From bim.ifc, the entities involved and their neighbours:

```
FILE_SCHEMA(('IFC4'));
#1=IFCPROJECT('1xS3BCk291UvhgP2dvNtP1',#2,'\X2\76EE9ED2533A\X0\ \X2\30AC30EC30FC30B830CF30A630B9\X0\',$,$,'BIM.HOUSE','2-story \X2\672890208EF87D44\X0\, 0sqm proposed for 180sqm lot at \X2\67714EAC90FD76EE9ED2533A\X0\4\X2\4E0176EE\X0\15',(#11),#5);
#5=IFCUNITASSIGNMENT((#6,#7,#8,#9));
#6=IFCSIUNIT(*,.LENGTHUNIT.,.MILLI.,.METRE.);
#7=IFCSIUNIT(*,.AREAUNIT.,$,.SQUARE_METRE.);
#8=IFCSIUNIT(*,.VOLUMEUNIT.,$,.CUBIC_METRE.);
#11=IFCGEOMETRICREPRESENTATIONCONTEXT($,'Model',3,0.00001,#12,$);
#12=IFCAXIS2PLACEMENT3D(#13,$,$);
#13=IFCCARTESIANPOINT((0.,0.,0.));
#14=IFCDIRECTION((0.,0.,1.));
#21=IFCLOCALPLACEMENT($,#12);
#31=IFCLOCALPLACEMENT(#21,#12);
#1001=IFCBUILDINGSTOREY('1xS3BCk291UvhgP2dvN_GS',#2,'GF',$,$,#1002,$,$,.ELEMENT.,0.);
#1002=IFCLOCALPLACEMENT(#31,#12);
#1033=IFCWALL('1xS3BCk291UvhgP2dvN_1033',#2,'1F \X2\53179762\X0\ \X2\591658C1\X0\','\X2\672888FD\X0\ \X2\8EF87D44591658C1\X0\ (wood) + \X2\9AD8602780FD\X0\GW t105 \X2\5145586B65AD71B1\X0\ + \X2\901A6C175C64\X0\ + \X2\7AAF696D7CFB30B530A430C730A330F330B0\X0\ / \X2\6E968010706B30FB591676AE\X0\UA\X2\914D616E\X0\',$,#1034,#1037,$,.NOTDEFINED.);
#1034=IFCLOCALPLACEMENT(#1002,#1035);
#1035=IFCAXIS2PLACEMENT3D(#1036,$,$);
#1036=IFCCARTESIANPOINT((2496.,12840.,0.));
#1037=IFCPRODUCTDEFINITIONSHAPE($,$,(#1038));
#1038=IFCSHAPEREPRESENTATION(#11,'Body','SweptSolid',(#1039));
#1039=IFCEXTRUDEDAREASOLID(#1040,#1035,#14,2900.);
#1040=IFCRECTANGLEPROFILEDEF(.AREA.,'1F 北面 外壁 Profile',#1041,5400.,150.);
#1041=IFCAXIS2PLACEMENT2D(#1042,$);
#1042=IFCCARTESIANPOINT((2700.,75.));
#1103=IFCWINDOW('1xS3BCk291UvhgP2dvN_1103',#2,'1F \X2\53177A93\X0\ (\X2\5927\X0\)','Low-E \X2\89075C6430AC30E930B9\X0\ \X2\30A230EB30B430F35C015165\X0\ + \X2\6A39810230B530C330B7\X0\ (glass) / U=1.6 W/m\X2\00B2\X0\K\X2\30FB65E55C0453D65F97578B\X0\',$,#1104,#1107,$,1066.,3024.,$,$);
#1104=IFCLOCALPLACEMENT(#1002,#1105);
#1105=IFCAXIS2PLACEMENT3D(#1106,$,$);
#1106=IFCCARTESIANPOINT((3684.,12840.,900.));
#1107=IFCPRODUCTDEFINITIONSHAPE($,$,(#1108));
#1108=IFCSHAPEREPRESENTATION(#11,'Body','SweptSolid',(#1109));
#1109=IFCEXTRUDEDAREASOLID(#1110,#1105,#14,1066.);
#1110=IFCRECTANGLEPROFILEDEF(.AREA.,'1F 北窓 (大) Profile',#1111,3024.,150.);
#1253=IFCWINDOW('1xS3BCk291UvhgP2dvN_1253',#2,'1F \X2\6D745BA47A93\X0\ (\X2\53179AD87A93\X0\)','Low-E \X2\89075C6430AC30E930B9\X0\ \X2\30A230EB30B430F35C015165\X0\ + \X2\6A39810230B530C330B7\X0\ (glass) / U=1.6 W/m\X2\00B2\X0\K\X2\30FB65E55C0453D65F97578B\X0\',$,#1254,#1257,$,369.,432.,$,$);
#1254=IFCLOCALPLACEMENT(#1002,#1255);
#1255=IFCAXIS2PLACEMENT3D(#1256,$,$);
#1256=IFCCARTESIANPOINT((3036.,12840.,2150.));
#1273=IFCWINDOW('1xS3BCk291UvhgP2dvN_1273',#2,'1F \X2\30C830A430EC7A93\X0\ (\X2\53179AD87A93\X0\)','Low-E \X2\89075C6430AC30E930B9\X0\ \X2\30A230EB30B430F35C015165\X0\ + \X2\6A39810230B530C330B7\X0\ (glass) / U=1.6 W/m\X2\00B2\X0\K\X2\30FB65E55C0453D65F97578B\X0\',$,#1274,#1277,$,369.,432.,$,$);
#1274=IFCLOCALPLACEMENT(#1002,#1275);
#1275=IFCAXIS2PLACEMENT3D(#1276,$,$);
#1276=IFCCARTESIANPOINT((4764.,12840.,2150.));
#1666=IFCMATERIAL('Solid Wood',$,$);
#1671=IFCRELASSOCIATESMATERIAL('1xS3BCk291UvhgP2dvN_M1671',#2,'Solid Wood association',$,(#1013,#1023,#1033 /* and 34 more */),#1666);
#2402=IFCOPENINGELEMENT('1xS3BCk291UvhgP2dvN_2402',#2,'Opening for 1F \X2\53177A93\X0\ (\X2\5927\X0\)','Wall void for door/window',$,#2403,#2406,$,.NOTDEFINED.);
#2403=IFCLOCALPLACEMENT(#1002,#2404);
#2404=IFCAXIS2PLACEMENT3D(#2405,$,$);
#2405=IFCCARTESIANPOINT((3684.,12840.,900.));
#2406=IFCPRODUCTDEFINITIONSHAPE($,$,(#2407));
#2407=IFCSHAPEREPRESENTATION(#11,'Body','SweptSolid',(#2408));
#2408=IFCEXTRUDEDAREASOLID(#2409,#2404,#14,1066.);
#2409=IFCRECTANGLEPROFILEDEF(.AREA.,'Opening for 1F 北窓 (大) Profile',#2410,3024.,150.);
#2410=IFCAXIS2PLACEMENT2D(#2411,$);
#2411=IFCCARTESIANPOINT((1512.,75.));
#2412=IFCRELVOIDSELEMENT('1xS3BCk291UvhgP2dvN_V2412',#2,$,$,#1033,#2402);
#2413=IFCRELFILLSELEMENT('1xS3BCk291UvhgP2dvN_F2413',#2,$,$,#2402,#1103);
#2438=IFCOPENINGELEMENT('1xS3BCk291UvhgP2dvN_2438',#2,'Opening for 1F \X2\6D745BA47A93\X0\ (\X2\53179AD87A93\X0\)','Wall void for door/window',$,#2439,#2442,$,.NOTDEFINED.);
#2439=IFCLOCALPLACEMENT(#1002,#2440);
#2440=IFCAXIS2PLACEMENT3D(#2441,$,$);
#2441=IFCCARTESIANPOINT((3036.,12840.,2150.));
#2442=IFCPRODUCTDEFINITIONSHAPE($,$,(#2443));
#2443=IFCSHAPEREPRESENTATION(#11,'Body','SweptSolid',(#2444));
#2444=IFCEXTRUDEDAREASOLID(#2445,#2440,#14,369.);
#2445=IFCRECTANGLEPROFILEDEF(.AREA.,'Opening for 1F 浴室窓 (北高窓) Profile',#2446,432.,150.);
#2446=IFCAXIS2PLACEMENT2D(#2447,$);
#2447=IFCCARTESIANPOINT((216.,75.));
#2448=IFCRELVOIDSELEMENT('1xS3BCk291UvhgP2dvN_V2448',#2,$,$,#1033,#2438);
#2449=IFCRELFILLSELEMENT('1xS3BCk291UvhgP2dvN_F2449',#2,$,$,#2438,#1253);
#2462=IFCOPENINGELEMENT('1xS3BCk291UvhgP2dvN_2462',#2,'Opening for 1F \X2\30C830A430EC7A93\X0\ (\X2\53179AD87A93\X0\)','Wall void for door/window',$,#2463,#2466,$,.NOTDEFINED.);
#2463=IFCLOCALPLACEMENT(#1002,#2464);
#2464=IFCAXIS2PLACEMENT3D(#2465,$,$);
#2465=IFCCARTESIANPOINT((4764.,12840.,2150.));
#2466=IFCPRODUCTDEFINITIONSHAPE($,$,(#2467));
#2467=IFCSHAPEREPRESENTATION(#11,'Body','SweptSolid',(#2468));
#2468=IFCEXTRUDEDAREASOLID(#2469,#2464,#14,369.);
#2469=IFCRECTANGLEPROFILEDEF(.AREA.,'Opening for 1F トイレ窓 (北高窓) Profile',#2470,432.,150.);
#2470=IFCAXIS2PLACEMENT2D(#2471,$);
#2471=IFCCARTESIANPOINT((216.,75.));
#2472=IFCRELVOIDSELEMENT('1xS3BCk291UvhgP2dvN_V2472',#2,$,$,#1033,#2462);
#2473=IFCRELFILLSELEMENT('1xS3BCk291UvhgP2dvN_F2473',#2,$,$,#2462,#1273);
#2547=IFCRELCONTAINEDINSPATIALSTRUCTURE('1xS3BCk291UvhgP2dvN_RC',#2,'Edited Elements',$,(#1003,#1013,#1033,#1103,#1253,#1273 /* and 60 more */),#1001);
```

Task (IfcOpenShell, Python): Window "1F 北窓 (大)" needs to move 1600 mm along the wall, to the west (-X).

```python
import ifcopenshell
import ifcopenshell.api.geometry
import ifcopenshell.util.placement
import ifcopenshell.util.unit

model = ifcopenshell.open("bim.ifc")
unit_scale = ifcopenshell.util.unit.calculate_unit_scale(model)

window = model.by_guid("1xS3BCk291UvhgP2dvN_1103")
opening = window.FillsVoids[0].RelatingOpeningElement
wall = opening.VoidsElements[0].RelatingBuildingElement

wall_matrix = ifcopenshell.util.placement.get_local_placement(wall.ObjectPlacement)
shift = wall_matrix[:3, 0] * -1.6 / unit_scale
before = ifcopenshell.util.placement.get_local_placement(window.ObjectPlacement)[:3, 3].copy()

# The window is not placed relative to its opening, so move both.
for product in (opening, window):
    matrix = ifcopenshell.util.placement.get_local_placement(product.ObjectPlacement)
    matrix[:3, 3] += shift
    ifcopenshell.api.geometry.edit_object_placement(model, product=product, matrix=matrix, is_si=False)

after = ifcopenshell.util.placement.get_local_placement(window.ObjectPlacement)[:3, 3]
print("window moved by", (after - before).round(3) + 0.0)

model.write("bim_rev.ifc")
```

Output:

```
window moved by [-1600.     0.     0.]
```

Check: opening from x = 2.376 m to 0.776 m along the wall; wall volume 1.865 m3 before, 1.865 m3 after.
